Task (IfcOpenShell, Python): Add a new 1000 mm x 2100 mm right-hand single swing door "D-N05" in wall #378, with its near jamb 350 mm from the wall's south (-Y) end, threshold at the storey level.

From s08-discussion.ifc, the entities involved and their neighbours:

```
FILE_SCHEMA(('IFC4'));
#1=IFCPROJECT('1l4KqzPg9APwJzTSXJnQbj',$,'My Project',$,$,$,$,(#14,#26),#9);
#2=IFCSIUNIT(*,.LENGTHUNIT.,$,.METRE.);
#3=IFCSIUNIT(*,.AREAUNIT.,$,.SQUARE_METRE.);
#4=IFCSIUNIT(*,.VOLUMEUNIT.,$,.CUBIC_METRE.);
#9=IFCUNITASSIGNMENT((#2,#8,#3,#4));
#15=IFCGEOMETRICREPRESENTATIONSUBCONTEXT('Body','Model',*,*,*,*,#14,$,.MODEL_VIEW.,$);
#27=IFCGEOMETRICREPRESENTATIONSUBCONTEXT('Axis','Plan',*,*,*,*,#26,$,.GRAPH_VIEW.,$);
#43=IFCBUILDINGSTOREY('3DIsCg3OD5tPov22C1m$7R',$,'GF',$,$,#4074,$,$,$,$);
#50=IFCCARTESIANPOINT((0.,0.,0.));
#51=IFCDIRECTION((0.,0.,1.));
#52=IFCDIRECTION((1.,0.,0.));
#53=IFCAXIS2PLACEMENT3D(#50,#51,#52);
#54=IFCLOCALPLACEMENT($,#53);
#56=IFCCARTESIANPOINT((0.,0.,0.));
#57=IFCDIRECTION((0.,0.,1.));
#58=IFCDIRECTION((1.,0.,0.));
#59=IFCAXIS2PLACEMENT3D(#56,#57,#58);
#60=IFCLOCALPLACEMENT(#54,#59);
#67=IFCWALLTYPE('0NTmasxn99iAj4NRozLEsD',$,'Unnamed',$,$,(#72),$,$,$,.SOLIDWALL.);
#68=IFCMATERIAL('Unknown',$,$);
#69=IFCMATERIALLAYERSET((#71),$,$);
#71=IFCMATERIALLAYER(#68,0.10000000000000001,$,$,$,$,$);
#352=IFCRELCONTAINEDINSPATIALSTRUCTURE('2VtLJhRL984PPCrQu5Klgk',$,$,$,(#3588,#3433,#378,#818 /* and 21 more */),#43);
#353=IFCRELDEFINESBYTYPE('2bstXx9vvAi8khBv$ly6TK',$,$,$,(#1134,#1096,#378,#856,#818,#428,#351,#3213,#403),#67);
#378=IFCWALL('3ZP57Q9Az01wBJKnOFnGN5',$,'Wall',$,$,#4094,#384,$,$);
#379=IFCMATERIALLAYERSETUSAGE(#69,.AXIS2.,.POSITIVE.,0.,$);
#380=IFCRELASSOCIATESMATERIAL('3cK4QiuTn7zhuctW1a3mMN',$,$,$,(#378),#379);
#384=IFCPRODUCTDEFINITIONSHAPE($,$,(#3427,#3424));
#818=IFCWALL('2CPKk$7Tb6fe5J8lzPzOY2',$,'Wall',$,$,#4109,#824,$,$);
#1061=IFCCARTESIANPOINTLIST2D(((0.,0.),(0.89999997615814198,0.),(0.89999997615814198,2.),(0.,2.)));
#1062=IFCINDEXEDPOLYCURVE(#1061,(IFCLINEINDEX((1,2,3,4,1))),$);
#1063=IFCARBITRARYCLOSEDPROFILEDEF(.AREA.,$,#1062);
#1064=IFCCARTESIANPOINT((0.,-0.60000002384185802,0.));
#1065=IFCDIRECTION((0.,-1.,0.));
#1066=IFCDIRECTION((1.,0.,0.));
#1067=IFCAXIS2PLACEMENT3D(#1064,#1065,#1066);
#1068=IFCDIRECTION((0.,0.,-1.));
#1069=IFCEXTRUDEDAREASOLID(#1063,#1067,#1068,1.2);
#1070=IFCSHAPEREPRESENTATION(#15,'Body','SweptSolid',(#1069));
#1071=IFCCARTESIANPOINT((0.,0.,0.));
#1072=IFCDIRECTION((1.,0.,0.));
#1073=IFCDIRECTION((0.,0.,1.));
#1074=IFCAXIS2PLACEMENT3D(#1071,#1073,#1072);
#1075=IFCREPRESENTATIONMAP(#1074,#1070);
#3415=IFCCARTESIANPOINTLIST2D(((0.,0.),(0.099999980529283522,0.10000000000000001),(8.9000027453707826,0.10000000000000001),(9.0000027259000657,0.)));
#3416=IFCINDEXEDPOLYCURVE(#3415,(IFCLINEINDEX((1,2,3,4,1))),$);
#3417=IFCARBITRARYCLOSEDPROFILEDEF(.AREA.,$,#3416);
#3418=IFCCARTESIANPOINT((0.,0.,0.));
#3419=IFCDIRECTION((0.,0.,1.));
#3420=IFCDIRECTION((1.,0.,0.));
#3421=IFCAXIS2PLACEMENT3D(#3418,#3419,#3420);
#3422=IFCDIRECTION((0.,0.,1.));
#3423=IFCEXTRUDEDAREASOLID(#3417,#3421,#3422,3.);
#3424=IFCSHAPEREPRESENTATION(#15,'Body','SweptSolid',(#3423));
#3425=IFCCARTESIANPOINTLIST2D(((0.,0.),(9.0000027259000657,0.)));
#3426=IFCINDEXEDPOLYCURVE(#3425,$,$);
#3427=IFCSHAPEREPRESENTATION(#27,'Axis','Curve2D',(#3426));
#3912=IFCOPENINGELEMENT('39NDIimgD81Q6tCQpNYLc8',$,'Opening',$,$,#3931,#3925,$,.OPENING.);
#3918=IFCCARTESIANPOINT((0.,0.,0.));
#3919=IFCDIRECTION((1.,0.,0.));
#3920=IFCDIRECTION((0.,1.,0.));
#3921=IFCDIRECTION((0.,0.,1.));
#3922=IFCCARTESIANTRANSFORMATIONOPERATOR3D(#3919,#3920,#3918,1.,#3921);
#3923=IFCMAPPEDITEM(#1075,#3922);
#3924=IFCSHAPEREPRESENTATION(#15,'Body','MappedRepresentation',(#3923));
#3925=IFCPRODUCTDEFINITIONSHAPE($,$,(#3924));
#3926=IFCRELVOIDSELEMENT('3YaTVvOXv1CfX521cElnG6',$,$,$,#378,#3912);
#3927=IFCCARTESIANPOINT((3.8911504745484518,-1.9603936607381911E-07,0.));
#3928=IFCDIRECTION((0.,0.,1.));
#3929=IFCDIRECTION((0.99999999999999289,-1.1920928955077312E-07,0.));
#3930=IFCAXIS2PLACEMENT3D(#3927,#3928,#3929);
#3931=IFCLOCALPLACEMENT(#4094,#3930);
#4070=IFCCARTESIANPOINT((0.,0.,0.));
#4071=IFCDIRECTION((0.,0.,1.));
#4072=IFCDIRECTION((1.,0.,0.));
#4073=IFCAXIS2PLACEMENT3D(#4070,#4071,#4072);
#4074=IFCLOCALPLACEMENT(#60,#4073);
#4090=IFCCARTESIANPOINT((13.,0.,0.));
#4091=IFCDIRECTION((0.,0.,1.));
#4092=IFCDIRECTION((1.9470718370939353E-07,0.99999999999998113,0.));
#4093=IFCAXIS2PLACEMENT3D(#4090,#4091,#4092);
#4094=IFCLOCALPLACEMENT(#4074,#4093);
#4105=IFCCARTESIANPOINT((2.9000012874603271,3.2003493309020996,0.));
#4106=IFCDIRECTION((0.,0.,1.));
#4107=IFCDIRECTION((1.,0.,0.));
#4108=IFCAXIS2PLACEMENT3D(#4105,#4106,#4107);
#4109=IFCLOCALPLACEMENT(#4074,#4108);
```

```python
import numpy as np
import ifcopenshell
import ifcopenshell.api.feature
import ifcopenshell.api.geometry
import ifcopenshell.api.root
import ifcopenshell.api.spatial
import ifcopenshell.geom
import ifcopenshell.util.element
import ifcopenshell.util.placement
import ifcopenshell.util.representation
import ifcopenshell.util.shape
import ifcopenshell.util.unit

model = ifcopenshell.open("s08-discussion.ifc")
unit_scale = ifcopenshell.util.unit.calculate_unit_scale(model)
settings = ifcopenshell.geom.settings()


def volume(element):
    """Net volume in cubic metres, openings subtracted."""
    shape = ifcopenshell.geom.create_shape(settings, element)
    return ifcopenshell.util.shape.get_volume(shape.geometry)


wall = model.by_guid("3ZP57Q9Az01wBJKnOFnGN5")
storey = ifcopenshell.util.element.get_container(wall, ifc_class="IfcBuildingStorey")
context = ifcopenshell.util.representation.get_context(model, "Model", "Body", "MODEL_VIEW")
before = volume(wall)

width, height, from_end, sill = 1, 2.1, 0.35, 0.0  # metres

# The wall runs along its own X axis, and the end named is its -X end.
wall_shape = ifcopenshell.geom.create_shape(settings, wall)
x, y, z = ifcopenshell.util.shape.get_vertices(wall_shape.geometry).T
start = x.min() + from_end
face, thickness = float(y.min()), float(y.max() - y.min())
wall_matrix = ifcopenshell.util.placement.get_local_placement(wall.ObjectPlacement)
level = ifcopenshell.util.placement.get_local_placement(storey.ObjectPlacement)[2, 3]


def in_wall(x, y):
    """Placement at x, y metres in the wall's axes, at sill height."""
    matrix = wall_matrix.copy()
    matrix[:, 3] = wall_matrix @ np.array([x / unit_scale, y / unit_scale, 0.0, 1.0])
    matrix[2, 3] = level + sill / unit_scale
    return matrix


# Opening: a box that overshoots both wall faces by 50 mm.
opening = ifcopenshell.api.root.create_entity(model, ifc_class="IfcOpeningElement", predefined_type="OPENING")
box = ifcopenshell.api.geometry.add_wall_representation(
    model, context=context, length=width, height=height, thickness=thickness + 0.1
)
ifcopenshell.api.geometry.assign_representation(model, product=opening, representation=box)
ifcopenshell.api.geometry.edit_object_placement(model, product=opening, matrix=in_wall(start, face - 0.05), is_si=False)
ifcopenshell.api.feature.add_feature(model, feature=opening, element=wall)

door = ifcopenshell.api.root.create_entity(model, ifc_class="IfcDoor", name="D-N05", predefined_type="DOOR")
door.OverallWidth, door.OverallHeight = width / unit_scale, height / unit_scale
door.OperationType = "SINGLE_SWING_RIGHT"
body = ifcopenshell.api.geometry.add_door_representation(
    model,
    context=context,
    overall_width=door.OverallWidth,
    overall_height=door.OverallHeight,
    operation_type="SINGLE_SWING_RIGHT",
    lining_properties={"LiningDepth": thickness / unit_scale, "ThresholdDepth": thickness / unit_scale},
)
ifcopenshell.api.geometry.assign_representation(model, product=door, representation=body)
ifcopenshell.api.spatial.assign_container(model, products=[door], relating_structure=storey)
ifcopenshell.api.feature.add_filling(model, opening=opening, element=door)

# The lining spans the wall, so the door starts at the wall face.
ifcopenshell.api.geometry.edit_object_placement(model, product=door, matrix=in_wall(start, face), is_si=False)

after = volume(wall)

print(f"wall volume {before:.3f} -> {after:.3f} m3")

model.write("s08-discussion_updated.ifc")
```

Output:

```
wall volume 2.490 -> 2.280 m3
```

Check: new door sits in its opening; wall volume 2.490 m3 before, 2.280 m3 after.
